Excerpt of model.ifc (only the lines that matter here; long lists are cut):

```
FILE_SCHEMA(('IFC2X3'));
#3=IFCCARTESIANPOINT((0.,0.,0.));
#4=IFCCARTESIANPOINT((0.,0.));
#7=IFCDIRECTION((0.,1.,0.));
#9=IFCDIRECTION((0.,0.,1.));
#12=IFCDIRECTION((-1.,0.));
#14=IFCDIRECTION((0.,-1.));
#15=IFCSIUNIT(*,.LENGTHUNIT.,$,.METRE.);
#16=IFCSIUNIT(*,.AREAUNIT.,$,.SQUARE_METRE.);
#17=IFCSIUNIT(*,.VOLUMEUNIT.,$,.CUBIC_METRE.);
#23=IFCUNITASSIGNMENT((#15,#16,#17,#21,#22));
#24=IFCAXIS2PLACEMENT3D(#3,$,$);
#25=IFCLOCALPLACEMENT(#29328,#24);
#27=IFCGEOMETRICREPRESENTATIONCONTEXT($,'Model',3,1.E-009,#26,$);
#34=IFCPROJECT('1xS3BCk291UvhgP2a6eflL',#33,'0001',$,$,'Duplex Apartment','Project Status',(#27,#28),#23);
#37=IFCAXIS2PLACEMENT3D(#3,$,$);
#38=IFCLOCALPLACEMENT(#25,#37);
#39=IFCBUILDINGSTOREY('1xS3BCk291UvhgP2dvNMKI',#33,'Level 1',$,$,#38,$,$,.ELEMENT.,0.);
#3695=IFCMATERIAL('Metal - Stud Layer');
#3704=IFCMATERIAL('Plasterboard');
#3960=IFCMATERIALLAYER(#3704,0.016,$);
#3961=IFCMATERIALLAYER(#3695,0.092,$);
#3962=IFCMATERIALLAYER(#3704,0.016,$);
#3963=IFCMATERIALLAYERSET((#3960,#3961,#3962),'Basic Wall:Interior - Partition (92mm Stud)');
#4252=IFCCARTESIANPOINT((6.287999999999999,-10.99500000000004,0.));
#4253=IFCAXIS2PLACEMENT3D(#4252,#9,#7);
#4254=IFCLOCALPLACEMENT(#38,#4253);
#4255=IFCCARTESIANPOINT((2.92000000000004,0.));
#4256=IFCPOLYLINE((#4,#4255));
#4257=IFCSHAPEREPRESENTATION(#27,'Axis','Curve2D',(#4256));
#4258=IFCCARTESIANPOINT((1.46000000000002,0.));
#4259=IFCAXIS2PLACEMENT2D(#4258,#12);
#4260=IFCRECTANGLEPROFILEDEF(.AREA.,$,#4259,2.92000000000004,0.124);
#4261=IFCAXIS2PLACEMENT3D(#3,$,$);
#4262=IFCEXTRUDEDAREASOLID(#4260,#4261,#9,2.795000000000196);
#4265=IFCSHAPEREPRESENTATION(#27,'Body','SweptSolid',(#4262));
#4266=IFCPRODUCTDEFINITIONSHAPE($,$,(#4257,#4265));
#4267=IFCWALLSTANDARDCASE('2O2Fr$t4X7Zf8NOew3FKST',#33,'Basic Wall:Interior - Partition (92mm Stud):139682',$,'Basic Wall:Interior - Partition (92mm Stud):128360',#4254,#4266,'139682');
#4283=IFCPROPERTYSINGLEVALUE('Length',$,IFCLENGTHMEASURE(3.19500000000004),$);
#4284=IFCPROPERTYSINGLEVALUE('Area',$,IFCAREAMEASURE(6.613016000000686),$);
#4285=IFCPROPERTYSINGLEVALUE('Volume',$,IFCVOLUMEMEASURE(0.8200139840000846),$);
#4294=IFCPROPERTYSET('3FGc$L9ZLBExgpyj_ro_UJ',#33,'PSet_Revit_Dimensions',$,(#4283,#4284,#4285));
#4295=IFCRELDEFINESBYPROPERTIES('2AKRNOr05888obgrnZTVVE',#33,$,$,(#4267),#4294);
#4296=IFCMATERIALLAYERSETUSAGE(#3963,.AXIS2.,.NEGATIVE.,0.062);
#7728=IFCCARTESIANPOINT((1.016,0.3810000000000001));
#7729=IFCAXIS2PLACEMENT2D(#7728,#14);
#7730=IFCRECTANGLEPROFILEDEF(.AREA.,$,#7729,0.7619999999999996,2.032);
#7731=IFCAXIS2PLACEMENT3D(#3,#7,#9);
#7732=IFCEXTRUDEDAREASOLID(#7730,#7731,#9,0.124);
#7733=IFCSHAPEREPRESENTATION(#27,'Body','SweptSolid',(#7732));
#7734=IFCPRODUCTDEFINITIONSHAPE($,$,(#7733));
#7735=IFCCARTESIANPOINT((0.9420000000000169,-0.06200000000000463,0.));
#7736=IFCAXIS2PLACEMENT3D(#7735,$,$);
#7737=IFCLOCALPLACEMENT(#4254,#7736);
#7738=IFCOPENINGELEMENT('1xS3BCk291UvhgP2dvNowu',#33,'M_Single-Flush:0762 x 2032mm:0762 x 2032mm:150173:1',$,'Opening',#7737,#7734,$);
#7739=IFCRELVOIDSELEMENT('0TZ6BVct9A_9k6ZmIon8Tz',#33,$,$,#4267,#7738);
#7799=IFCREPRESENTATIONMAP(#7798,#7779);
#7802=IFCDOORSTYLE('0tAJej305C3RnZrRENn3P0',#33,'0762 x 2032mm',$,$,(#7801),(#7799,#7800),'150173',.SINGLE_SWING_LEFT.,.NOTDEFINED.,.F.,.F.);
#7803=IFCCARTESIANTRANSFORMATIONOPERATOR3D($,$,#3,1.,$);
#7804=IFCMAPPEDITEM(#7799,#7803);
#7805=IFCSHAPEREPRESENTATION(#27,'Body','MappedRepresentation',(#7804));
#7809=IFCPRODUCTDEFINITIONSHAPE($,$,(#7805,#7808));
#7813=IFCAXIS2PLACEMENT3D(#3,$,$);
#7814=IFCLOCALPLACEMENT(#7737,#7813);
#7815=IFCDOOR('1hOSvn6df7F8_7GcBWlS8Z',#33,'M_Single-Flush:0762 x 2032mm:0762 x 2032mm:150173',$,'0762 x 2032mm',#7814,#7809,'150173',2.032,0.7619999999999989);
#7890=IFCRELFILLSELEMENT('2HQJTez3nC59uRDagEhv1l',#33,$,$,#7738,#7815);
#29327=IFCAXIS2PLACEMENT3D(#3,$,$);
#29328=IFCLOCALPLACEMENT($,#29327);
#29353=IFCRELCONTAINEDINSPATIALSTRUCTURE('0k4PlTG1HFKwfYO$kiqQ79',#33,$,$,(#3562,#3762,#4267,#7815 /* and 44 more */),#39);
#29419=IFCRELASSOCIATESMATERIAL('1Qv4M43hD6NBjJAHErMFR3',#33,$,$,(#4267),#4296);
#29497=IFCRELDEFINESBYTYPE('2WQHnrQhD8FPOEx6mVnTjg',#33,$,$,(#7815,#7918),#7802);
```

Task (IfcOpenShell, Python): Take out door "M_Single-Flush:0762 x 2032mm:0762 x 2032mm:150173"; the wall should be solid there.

```python
import ifcopenshell
import ifcopenshell.api.feature
import ifcopenshell.api.pset
import ifcopenshell.api.root
import ifcopenshell.geom
import ifcopenshell.util.element
import ifcopenshell.util.shape
import ifcopenshell.util.unit

model = ifcopenshell.open("model.ifc")
area_scale = ifcopenshell.util.unit.calculate_unit_scale(model, "AREAUNIT")
volume_scale = ifcopenshell.util.unit.calculate_unit_scale(model, "VOLUMEUNIT")
settings = ifcopenshell.geom.settings()


def volume(element):
    """Net volume in cubic metres, openings subtracted."""
    shape = ifcopenshell.geom.create_shape(settings, element)
    return ifcopenshell.util.shape.get_volume(shape.geometry)


door = model.by_guid("1hOSvn6df7F8_7GcBWlS8Z")
opening = door.FillsVoids[0].RelatingOpeningElement
wall = opening.VoidsElements[0].RelatingBuildingElement
before = volume(wall)

ifcopenshell.api.root.remove_product(model, product=door)
ifcopenshell.api.feature.remove_feature(model, feature=opening)

after = volume(wall)
thickness = 0.124  # wall thickness in metres

# Update the wall's stored quantities.
pset = model.by_id(ifcopenshell.util.element.get_pset(wall, "PSet_Revit_Dimensions", should_inherit=False)["id"])
ifcopenshell.api.pset.edit_pset(model, pset=pset, properties={
    "Area": model.create_entity("IfcAreaMeasure", after / thickness / area_scale),
    "Volume": model.create_entity("IfcVolumeMeasure", after / volume_scale),
})

print(f"wall volume {before:.3f} -> {after:.3f} m3")

model.write("model_v2.ifc")
```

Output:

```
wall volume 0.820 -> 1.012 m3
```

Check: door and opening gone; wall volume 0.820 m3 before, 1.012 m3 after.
